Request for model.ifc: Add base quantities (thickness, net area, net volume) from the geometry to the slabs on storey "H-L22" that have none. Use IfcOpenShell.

First a look at what the model holds.

```python
import ifcopenshell
import ifcopenshell.util.element
import ifcopenshell.util.unit

model = ifcopenshell.open("model.ifc")
print(model.schema)
for unit_type in ("LENGTHUNIT", "AREAUNIT", "VOLUMEUNIT"):
    print(unit_type, ifcopenshell.util.unit.calculate_unit_scale(model, unit_type))
storey = next(s for s in model.by_type("IfcBuildingStorey") if s.Name == "H-L22")
slabs = [e for e in ifcopenshell.util.element.get_decomposition(storey) if e.is_a("IfcSlab")]
for e in sorted(slabs, key=lambda e: e.id()):
    print(e.id(), e.is_a(), e.Name, list(ifcopenshell.util.element.get_psets(e, qtos_only=True)), sep=" | ")
```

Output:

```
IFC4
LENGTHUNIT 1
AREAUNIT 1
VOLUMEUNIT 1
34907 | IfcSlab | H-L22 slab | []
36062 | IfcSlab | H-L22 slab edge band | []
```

```python
import ifcopenshell
import ifcopenshell.api.pset
import ifcopenshell.geom
import ifcopenshell.util.element
import ifcopenshell.util.shape
import ifcopenshell.util.unit

model = ifcopenshell.open("model.ifc")
unit_scale = ifcopenshell.util.unit.calculate_unit_scale(model)
area_scale = ifcopenshell.util.unit.calculate_unit_scale(model, "AREAUNIT")
volume_scale = ifcopenshell.util.unit.calculate_unit_scale(model, "VOLUMEUNIT")
settings = ifcopenshell.geom.settings()

storey = next(s for s in model.by_type("IfcBuildingStorey") if s.Name == "H-L22")
slabs = [e for e in ifcopenshell.util.element.get_decomposition(storey) if e.is_a("IfcSlab")]

for e in sorted(slabs, key=lambda e: e.id()):
    if ifcopenshell.util.element.get_psets(e, qtos_only=True, should_inherit=False):
        continue
    # Geometry comes back in metres, in the element's own axes.
    shape = ifcopenshell.geom.create_shape(settings, e)
    values = {
        "Width": ifcopenshell.util.shape.get_z(shape.geometry) / unit_scale,
        "NetArea": ifcopenshell.util.shape.get_footprint_area(shape.geometry) / area_scale,
        "NetVolume": ifcopenshell.util.shape.get_volume(shape.geometry) / volume_scale,
    }
    qto = ifcopenshell.api.pset.add_qto(model, product=e, name="Qto_SlabBaseQuantities")
    ifcopenshell.api.pset.edit_qto(model, qto=qto, properties=values)
    print(e.id(), {k: round(v, 3) for k, v in values.items()})

model.write("model_rev.ifc")
```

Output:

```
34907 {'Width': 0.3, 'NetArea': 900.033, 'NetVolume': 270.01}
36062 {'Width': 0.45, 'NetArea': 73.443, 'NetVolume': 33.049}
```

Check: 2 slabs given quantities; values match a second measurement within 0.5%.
